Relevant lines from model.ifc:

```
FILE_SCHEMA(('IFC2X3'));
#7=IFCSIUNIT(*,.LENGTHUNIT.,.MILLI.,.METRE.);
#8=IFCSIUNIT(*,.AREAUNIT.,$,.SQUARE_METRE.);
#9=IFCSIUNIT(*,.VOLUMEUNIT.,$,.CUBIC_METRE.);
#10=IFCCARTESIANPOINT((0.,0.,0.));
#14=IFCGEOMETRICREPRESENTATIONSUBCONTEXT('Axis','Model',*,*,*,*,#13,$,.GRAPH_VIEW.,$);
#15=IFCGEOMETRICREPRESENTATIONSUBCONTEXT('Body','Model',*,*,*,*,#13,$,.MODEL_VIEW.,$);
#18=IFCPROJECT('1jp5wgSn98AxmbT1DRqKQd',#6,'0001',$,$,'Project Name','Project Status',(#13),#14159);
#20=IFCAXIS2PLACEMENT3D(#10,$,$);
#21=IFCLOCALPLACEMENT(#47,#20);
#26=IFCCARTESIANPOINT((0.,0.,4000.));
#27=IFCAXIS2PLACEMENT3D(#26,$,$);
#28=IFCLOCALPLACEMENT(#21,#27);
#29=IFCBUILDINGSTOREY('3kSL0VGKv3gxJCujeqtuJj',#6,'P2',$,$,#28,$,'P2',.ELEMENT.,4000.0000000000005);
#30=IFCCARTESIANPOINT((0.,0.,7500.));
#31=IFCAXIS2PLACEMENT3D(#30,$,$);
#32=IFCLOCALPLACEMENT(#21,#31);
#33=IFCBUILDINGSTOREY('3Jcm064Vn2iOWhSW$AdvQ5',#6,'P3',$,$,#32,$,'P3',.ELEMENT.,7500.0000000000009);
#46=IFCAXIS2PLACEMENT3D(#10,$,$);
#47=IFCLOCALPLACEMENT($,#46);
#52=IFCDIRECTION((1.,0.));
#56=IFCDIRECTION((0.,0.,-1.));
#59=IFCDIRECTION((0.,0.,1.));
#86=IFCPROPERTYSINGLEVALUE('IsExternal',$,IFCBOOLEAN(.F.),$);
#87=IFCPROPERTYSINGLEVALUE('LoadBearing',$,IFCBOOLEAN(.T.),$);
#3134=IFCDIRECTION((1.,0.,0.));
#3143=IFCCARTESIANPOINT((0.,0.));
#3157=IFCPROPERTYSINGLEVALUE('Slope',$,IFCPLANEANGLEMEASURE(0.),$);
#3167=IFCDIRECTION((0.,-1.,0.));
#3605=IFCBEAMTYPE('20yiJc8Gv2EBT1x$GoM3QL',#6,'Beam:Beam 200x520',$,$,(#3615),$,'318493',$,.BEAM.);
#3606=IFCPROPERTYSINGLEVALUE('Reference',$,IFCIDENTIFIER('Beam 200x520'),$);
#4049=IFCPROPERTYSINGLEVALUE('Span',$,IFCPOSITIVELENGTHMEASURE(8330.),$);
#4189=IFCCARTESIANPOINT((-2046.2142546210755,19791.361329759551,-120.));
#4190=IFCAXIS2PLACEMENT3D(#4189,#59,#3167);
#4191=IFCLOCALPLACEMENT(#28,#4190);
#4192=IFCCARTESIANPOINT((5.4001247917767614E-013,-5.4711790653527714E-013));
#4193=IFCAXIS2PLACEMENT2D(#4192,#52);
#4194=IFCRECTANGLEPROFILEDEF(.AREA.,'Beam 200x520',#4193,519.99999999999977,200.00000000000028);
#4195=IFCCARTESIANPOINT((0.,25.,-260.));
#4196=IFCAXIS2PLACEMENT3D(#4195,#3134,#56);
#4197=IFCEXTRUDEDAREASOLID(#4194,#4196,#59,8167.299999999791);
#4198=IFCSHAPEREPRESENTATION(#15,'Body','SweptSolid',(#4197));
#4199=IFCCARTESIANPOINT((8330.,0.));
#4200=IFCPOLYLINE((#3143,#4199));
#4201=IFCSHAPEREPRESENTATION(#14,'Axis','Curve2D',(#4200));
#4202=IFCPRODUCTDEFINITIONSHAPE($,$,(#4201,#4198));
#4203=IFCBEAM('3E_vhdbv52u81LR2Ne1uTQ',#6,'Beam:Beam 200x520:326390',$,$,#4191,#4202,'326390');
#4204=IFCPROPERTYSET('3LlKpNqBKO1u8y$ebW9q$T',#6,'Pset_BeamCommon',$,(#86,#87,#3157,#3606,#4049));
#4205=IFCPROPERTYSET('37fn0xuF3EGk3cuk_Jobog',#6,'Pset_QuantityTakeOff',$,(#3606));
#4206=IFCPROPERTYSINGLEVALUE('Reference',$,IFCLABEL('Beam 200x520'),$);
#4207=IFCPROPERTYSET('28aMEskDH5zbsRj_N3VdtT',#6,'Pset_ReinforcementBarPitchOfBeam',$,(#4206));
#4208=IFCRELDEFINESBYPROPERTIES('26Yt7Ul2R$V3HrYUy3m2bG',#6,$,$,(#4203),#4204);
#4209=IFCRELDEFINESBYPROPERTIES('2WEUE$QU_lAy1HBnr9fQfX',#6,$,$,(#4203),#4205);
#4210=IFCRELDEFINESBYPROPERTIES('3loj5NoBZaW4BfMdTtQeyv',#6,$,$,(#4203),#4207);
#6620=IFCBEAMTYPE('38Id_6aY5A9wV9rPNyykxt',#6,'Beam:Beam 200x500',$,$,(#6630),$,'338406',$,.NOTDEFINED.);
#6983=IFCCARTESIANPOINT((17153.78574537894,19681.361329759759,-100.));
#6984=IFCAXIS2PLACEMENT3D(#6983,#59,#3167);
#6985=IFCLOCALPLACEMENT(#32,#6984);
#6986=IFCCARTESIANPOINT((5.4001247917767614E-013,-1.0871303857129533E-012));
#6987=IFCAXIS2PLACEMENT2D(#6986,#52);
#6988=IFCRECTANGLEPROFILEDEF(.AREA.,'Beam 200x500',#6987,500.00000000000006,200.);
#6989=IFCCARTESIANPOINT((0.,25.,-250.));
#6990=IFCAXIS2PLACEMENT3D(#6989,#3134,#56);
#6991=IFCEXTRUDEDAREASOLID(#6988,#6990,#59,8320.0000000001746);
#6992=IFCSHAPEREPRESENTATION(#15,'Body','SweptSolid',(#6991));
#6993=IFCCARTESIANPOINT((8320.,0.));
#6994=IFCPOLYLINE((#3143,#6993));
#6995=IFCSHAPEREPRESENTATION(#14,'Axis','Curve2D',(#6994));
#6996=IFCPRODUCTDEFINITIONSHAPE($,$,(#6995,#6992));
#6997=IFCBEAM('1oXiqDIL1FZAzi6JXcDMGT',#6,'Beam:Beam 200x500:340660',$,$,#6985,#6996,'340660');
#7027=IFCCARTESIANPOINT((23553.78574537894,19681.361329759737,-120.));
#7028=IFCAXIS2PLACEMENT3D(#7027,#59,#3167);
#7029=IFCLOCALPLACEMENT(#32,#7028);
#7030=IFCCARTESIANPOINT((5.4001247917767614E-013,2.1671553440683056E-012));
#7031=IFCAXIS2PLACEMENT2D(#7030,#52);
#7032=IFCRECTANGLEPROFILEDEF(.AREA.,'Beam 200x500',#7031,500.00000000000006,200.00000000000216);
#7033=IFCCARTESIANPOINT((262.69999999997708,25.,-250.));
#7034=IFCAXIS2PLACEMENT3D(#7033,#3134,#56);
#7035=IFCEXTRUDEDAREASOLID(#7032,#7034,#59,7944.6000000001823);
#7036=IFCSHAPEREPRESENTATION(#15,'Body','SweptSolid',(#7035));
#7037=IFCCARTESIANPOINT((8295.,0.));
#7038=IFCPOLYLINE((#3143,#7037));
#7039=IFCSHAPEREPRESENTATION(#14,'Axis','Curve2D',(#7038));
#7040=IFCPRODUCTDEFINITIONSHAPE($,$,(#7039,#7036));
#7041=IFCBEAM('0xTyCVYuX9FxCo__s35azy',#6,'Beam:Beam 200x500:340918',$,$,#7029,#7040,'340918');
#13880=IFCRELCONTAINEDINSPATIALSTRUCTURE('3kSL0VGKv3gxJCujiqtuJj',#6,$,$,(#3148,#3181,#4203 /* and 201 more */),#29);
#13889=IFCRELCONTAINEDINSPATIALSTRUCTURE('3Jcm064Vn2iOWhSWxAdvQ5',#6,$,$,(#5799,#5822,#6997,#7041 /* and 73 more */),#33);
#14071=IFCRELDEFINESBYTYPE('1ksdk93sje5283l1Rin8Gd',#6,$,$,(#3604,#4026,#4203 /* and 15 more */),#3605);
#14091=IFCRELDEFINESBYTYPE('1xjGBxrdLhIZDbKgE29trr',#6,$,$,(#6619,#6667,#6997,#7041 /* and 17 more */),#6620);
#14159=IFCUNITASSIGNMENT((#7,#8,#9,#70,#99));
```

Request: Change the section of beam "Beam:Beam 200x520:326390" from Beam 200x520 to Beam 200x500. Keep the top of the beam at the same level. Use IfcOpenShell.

```python
import ifcopenshell
import ifcopenshell.api.pset
import ifcopenshell.api.type
import ifcopenshell.util.element
import ifcopenshell.util.representation

model = ifcopenshell.open("model.ifc")

member = model.by_id(4203)
source = next(p for p in model.by_type("IfcRectangleProfileDef") if p.ProfileName == "Beam 200x500")

body = ifcopenshell.util.representation.get_representation(member, "Model", "Body")
solid = body.Items[0]
old_profile = solid.SweptArea

# Copy the section's sizes but keep this member's own profile position.
profile = ifcopenshell.util.element.copy(model, source)
# Profiles are centred, so shift by half the change in depth to hold the top.
shift = (old_profile.XDim - profile.XDim) / 2
x, y = old_profile.Position.Location.Coordinates
up = (-1.0, 0.0)  # upwards, in the solid's own plane
location = model.createIfcCartesianPoint((x + up[0] * shift, y + up[1] * shift))
profile.Position = model.createIfcAxis2Placement2D(location, old_profile.Position.RefDirection)
solid.SweptArea = profile
if not model.get_total_inverses(old_profile):
    ifcopenshell.util.element.remove_deep2(model, old_profile)

new_type = model.by_guid("38Id_6aY5A9wV9rPNyykxt")
ifcopenshell.api.type.assign_type(
    model, related_objects=[member], relating_type=new_type, should_map_representations=False
)
member.Name = member.Name.replace("Beam 200x520", "Beam 200x500")
pset = model.by_id(ifcopenshell.util.element.get_pset(member, "Pset_BeamCommon", should_inherit=False)["id"])
ifcopenshell.api.pset.edit_pset(model, pset=pset, properties={"Reference": "Beam 200x500"})
pset = model.by_id(ifcopenshell.util.element.get_pset(member, "Pset_QuantityTakeOff", should_inherit=False)["id"])
ifcopenshell.api.pset.edit_pset(model, pset=pset, properties={"Reference": "Beam 200x500"})
pset = model.by_id(ifcopenshell.util.element.get_pset(member, "Pset_ReinforcementBarPitchOfBeam", should_inherit=False)["id"])
ifcopenshell.api.pset.edit_pset(model, pset=pset, properties={"Reference": "Beam 200x500"})

print(solid.SweptArea)

model.write("model-out.ifc")
```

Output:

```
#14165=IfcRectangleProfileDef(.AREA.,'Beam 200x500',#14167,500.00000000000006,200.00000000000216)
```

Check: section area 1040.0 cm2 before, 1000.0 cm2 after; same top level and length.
